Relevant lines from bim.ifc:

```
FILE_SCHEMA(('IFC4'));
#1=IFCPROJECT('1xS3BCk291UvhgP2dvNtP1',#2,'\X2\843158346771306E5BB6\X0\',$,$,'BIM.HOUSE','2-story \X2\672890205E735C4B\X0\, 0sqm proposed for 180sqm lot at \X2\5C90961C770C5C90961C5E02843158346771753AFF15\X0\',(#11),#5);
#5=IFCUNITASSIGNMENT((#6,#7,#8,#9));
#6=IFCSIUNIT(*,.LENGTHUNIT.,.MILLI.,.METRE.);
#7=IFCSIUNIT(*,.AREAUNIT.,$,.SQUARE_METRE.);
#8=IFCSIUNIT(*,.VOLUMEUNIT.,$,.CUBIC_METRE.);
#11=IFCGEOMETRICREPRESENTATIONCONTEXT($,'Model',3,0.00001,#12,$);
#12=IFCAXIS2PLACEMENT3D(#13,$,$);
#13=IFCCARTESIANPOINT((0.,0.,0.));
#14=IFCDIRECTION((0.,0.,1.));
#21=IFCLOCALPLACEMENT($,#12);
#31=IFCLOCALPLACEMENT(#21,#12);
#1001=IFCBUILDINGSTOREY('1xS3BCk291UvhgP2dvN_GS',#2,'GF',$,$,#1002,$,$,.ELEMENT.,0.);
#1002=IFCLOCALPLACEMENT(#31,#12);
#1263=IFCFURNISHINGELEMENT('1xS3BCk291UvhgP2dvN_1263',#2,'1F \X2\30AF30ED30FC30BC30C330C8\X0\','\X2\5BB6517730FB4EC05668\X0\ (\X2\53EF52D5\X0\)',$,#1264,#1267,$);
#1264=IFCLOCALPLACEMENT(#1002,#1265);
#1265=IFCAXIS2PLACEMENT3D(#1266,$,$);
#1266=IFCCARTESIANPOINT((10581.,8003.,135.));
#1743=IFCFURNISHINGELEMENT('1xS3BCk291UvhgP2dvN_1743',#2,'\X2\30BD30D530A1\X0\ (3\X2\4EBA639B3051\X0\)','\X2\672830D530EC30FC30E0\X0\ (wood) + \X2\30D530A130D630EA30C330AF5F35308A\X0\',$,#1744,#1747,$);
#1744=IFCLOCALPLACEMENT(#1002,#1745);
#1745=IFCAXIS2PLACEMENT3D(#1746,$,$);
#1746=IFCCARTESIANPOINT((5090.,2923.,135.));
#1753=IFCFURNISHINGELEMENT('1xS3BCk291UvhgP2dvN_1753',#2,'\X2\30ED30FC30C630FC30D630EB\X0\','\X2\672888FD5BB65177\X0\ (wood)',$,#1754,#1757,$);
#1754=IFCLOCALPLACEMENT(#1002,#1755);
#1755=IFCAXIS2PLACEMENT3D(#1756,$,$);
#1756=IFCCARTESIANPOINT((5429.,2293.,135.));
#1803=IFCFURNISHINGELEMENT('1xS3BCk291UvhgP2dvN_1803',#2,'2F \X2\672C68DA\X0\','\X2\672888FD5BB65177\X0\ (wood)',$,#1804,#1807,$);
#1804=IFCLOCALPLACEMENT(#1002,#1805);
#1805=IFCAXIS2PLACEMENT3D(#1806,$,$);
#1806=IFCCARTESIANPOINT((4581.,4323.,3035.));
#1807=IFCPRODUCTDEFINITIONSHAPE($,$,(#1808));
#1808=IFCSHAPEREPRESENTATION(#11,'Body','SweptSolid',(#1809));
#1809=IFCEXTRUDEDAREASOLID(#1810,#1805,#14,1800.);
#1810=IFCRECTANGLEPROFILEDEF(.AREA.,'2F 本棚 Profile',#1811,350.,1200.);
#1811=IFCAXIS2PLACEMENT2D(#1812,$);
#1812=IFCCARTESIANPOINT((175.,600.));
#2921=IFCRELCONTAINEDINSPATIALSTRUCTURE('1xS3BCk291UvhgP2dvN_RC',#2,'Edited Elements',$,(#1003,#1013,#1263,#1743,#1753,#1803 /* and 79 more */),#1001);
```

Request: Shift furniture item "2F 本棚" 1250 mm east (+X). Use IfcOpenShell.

```python
import ifcopenshell
import ifcopenshell.api.geometry
import ifcopenshell.util.placement
import ifcopenshell.util.unit

model = ifcopenshell.open("bim.ifc")
unit_scale = ifcopenshell.util.unit.calculate_unit_scale(model)

item = model.by_guid("1xS3BCk291UvhgP2dvN_1803")
matrix = ifcopenshell.util.placement.get_local_placement(item.ObjectPlacement)
matrix[0, 3] += 1.25 / unit_scale
ifcopenshell.api.geometry.edit_object_placement(model, product=item, matrix=matrix, is_si=False)

print(ifcopenshell.util.placement.get_local_placement(item.ObjectPlacement).round(3) + 0.0)

model.write("bim_v2.ifc")
```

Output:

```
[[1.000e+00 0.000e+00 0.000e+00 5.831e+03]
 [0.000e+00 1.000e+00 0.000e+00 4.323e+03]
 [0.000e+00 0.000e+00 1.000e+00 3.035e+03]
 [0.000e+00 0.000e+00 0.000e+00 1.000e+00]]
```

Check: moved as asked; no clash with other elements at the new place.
